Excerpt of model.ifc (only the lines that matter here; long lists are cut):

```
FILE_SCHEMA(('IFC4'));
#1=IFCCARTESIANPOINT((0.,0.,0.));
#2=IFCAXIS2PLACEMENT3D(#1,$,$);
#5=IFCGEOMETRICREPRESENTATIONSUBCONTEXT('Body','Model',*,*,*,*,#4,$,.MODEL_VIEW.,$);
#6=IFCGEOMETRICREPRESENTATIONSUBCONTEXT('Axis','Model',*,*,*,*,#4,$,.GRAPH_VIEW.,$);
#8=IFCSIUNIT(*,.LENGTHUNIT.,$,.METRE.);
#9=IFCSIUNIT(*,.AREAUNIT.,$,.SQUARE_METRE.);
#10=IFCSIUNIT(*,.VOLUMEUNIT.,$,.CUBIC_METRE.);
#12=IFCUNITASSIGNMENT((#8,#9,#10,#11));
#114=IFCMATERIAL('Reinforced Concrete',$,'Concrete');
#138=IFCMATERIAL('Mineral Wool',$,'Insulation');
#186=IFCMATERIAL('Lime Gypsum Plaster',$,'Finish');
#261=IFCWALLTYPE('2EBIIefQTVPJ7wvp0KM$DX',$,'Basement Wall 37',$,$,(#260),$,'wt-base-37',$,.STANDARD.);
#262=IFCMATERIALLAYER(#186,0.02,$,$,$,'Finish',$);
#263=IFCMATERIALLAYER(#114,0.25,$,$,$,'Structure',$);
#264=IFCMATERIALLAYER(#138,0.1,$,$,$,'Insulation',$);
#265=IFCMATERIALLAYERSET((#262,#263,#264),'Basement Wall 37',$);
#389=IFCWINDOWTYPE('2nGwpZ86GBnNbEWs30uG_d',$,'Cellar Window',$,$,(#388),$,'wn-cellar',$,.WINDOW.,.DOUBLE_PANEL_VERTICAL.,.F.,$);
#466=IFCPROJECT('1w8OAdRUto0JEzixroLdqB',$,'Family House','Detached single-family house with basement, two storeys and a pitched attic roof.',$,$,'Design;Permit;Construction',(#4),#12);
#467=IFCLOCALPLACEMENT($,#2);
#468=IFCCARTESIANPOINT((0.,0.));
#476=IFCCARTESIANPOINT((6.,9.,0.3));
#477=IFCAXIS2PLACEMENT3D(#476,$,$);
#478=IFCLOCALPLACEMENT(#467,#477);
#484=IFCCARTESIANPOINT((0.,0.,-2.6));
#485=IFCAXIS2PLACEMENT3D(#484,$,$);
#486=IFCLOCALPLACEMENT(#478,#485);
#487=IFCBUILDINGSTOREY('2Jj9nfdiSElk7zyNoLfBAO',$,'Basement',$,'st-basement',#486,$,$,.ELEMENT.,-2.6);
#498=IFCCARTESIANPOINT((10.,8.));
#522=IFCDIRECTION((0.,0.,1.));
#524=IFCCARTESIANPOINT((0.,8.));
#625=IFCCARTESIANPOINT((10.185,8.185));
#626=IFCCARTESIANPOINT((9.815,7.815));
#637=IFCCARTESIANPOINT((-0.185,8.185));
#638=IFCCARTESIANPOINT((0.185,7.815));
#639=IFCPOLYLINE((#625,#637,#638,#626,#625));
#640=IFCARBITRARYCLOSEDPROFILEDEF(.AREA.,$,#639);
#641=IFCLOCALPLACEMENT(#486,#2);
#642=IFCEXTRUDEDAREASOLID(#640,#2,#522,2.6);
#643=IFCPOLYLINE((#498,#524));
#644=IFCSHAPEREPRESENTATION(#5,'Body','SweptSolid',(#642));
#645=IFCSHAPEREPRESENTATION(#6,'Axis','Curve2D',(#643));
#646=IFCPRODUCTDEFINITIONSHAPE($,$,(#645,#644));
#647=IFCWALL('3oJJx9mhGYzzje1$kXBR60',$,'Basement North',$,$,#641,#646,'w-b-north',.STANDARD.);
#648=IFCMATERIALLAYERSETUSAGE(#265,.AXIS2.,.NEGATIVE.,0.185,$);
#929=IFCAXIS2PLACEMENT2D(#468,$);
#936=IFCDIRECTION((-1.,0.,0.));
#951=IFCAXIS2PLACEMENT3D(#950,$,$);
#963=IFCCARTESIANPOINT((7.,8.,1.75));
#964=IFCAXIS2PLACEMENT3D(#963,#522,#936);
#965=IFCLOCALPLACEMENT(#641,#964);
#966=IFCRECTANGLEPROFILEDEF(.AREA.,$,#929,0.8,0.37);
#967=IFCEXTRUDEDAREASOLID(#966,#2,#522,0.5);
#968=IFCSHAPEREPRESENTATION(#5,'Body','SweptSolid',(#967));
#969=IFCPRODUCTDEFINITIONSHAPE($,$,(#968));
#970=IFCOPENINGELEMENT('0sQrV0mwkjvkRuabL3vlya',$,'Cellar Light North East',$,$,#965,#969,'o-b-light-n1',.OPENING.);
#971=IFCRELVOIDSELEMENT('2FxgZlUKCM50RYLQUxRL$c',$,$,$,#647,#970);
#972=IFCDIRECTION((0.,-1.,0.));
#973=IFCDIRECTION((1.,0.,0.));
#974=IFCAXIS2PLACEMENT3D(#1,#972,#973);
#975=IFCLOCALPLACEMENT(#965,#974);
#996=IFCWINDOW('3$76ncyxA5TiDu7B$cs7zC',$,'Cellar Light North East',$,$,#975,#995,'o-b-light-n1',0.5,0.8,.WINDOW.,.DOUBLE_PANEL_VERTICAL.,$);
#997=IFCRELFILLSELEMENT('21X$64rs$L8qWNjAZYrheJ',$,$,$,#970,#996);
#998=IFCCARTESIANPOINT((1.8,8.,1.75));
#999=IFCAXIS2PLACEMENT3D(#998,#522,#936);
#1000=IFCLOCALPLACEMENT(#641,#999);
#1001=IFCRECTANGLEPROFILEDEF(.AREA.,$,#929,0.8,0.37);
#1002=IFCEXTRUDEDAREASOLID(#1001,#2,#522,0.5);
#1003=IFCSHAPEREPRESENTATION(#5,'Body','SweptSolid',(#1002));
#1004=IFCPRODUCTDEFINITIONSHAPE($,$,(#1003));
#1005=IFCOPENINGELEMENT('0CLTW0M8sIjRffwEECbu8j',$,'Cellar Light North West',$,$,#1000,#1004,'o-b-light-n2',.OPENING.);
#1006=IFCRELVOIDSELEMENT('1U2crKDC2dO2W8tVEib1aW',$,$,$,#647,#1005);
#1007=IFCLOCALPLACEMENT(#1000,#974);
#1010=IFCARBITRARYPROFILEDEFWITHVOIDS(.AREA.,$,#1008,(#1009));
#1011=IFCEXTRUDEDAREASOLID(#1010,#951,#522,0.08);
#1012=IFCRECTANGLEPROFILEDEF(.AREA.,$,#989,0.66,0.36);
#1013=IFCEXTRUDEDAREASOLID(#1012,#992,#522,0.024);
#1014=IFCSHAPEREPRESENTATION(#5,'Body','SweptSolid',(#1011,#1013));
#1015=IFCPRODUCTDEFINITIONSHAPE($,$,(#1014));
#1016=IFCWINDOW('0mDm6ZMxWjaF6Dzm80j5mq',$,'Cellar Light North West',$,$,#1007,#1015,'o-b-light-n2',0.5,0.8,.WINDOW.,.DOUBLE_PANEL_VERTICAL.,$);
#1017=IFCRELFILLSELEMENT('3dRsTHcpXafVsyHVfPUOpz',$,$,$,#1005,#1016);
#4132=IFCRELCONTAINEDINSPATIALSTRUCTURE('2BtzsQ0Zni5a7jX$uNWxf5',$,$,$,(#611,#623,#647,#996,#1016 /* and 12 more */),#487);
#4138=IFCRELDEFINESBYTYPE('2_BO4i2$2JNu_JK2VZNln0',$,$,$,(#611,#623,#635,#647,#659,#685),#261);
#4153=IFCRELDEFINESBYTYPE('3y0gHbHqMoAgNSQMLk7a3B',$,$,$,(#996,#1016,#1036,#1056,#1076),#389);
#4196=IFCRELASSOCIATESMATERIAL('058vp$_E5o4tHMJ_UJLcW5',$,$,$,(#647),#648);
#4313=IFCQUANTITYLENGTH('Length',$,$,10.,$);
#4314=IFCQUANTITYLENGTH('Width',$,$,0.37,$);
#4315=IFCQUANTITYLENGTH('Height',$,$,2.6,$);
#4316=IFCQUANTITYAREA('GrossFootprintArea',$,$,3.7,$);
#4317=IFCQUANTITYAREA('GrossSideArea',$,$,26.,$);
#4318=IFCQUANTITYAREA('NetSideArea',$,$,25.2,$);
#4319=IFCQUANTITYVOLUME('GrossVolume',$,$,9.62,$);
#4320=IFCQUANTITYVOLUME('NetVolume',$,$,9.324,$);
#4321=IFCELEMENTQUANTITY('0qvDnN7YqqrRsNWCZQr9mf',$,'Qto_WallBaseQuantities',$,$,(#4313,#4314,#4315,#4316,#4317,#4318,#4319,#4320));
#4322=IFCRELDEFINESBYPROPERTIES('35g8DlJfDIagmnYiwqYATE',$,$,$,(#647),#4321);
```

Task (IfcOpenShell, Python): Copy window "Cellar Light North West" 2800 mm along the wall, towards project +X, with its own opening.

```python
import ifcopenshell
import ifcopenshell.api.feature
import ifcopenshell.api.geometry
import ifcopenshell.api.pset
import ifcopenshell.api.root
import ifcopenshell.geom
import ifcopenshell.util.element
import ifcopenshell.util.placement
import ifcopenshell.util.shape
import ifcopenshell.util.unit

model = ifcopenshell.open("model.ifc")
unit_scale = ifcopenshell.util.unit.calculate_unit_scale(model)
area_scale = ifcopenshell.util.unit.calculate_unit_scale(model, "AREAUNIT")
volume_scale = ifcopenshell.util.unit.calculate_unit_scale(model, "VOLUMEUNIT")
settings = ifcopenshell.geom.settings()


def volume(element):
    """Net volume in cubic metres, openings subtracted."""
    shape = ifcopenshell.geom.create_shape(settings, element)
    return ifcopenshell.util.shape.get_volume(shape.geometry)


window = model.by_guid("0mDm6ZMxWjaF6Dzm80j5mq")
opening = window.FillsVoids[0].RelatingOpeningElement
wall = opening.VoidsElements[0].RelatingBuildingElement
before = volume(wall)
shift = ifcopenshell.util.placement.get_local_placement(wall.ObjectPlacement)[:3, 0] * 2.8 / unit_scale

# copy_class copies the void relationship, type, container and properties, but no geometry.
new_opening = ifcopenshell.api.root.copy_class(model, product=opening)
new_opening.Representation = ifcopenshell.util.element.copy_deep(
    model, opening.Representation, exclude=["IfcGeometricRepresentationContext", "IfcRepresentationMap"]
)
new_opening.Tag = None
new_window = ifcopenshell.api.root.copy_class(model, product=window)
new_window.Representation = ifcopenshell.util.element.copy_deep(
    model, window.Representation, exclude=["IfcGeometricRepresentationContext", "IfcRepresentationMap"]
)
new_window.Tag = None
ifcopenshell.api.feature.add_filling(model, opening=new_opening, element=new_window)

for old, new in ((opening, new_opening), (window, new_window)):
    matrix = ifcopenshell.util.placement.get_local_placement(old.ObjectPlacement)
    matrix[:3, 3] += shift
    ifcopenshell.api.geometry.edit_object_placement(model, product=new, matrix=matrix, is_si=False)

after = volume(wall)
thickness = 0.37  # wall thickness in metres

# Update the wall's stored quantities.
qto = model.by_id(ifcopenshell.util.element.get_pset(wall, "Qto_WallBaseQuantities", should_inherit=False)["id"])
ifcopenshell.api.pset.edit_qto(model, qto=qto, properties={
    "NetSideArea": after / thickness / area_scale,
    "NetVolume": after / volume_scale,
})

print(f"wall volume {before:.3f} -> {after:.3f} m3")

model.write("model-out.ifc")
```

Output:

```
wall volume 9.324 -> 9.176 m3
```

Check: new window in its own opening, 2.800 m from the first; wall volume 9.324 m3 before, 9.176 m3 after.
